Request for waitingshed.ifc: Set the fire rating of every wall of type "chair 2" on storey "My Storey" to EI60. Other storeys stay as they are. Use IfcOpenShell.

First a look at what the model holds.

```python
import ifcopenshell
import ifcopenshell.util.element

model = ifcopenshell.open("waitingshed.ifc")
print(model.schema)
storey = next(s for s in model.by_type("IfcBuildingStorey") if s.Name == "My Storey")
walls = [e for e in ifcopenshell.util.element.get_decomposition(storey) if e.is_a("IfcWall")]
seen = {}
for e in walls:
    element_type = ifcopenshell.util.element.get_type(e)
    key = (element_type.Name if element_type != e and element_type else None, ifcopenshell.util.element.get_pset(e, "Pset_WallCommon", "FireRating"))
    seen[key] = seen.get(key, 0) + 1
for (name, value), count in sorted(seen.items(), key=str):
    print(count, "x", name, "|", value)
```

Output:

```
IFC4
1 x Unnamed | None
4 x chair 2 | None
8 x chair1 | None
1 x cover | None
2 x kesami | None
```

```python
import ifcopenshell
import ifcopenshell.api.pset
import ifcopenshell.util.element

model = ifcopenshell.open("waitingshed.ifc")

storey = next(s for s in model.by_type("IfcBuildingStorey") if s.Name == "My Storey")
walls = [e for e in ifcopenshell.util.element.get_decomposition(storey) if e.is_a("IfcWall")]

count = 0
for e in walls:
    element_type = ifcopenshell.util.element.get_type(e)
    if element_type in (None, e) or element_type.Name != "chair 2":
        continue
    # add_pset returns the element's existing set when there is one.
    pset = ifcopenshell.api.pset.add_pset(model, product=e, name="Pset_WallCommon")
    ifcopenshell.api.pset.edit_pset(model, pset=pset, properties={"FireRating": "EI60"})
    count += 1

print(count, "walls updated")

model.write("waitingshed_v2.ifc")
```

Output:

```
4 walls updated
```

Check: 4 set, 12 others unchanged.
